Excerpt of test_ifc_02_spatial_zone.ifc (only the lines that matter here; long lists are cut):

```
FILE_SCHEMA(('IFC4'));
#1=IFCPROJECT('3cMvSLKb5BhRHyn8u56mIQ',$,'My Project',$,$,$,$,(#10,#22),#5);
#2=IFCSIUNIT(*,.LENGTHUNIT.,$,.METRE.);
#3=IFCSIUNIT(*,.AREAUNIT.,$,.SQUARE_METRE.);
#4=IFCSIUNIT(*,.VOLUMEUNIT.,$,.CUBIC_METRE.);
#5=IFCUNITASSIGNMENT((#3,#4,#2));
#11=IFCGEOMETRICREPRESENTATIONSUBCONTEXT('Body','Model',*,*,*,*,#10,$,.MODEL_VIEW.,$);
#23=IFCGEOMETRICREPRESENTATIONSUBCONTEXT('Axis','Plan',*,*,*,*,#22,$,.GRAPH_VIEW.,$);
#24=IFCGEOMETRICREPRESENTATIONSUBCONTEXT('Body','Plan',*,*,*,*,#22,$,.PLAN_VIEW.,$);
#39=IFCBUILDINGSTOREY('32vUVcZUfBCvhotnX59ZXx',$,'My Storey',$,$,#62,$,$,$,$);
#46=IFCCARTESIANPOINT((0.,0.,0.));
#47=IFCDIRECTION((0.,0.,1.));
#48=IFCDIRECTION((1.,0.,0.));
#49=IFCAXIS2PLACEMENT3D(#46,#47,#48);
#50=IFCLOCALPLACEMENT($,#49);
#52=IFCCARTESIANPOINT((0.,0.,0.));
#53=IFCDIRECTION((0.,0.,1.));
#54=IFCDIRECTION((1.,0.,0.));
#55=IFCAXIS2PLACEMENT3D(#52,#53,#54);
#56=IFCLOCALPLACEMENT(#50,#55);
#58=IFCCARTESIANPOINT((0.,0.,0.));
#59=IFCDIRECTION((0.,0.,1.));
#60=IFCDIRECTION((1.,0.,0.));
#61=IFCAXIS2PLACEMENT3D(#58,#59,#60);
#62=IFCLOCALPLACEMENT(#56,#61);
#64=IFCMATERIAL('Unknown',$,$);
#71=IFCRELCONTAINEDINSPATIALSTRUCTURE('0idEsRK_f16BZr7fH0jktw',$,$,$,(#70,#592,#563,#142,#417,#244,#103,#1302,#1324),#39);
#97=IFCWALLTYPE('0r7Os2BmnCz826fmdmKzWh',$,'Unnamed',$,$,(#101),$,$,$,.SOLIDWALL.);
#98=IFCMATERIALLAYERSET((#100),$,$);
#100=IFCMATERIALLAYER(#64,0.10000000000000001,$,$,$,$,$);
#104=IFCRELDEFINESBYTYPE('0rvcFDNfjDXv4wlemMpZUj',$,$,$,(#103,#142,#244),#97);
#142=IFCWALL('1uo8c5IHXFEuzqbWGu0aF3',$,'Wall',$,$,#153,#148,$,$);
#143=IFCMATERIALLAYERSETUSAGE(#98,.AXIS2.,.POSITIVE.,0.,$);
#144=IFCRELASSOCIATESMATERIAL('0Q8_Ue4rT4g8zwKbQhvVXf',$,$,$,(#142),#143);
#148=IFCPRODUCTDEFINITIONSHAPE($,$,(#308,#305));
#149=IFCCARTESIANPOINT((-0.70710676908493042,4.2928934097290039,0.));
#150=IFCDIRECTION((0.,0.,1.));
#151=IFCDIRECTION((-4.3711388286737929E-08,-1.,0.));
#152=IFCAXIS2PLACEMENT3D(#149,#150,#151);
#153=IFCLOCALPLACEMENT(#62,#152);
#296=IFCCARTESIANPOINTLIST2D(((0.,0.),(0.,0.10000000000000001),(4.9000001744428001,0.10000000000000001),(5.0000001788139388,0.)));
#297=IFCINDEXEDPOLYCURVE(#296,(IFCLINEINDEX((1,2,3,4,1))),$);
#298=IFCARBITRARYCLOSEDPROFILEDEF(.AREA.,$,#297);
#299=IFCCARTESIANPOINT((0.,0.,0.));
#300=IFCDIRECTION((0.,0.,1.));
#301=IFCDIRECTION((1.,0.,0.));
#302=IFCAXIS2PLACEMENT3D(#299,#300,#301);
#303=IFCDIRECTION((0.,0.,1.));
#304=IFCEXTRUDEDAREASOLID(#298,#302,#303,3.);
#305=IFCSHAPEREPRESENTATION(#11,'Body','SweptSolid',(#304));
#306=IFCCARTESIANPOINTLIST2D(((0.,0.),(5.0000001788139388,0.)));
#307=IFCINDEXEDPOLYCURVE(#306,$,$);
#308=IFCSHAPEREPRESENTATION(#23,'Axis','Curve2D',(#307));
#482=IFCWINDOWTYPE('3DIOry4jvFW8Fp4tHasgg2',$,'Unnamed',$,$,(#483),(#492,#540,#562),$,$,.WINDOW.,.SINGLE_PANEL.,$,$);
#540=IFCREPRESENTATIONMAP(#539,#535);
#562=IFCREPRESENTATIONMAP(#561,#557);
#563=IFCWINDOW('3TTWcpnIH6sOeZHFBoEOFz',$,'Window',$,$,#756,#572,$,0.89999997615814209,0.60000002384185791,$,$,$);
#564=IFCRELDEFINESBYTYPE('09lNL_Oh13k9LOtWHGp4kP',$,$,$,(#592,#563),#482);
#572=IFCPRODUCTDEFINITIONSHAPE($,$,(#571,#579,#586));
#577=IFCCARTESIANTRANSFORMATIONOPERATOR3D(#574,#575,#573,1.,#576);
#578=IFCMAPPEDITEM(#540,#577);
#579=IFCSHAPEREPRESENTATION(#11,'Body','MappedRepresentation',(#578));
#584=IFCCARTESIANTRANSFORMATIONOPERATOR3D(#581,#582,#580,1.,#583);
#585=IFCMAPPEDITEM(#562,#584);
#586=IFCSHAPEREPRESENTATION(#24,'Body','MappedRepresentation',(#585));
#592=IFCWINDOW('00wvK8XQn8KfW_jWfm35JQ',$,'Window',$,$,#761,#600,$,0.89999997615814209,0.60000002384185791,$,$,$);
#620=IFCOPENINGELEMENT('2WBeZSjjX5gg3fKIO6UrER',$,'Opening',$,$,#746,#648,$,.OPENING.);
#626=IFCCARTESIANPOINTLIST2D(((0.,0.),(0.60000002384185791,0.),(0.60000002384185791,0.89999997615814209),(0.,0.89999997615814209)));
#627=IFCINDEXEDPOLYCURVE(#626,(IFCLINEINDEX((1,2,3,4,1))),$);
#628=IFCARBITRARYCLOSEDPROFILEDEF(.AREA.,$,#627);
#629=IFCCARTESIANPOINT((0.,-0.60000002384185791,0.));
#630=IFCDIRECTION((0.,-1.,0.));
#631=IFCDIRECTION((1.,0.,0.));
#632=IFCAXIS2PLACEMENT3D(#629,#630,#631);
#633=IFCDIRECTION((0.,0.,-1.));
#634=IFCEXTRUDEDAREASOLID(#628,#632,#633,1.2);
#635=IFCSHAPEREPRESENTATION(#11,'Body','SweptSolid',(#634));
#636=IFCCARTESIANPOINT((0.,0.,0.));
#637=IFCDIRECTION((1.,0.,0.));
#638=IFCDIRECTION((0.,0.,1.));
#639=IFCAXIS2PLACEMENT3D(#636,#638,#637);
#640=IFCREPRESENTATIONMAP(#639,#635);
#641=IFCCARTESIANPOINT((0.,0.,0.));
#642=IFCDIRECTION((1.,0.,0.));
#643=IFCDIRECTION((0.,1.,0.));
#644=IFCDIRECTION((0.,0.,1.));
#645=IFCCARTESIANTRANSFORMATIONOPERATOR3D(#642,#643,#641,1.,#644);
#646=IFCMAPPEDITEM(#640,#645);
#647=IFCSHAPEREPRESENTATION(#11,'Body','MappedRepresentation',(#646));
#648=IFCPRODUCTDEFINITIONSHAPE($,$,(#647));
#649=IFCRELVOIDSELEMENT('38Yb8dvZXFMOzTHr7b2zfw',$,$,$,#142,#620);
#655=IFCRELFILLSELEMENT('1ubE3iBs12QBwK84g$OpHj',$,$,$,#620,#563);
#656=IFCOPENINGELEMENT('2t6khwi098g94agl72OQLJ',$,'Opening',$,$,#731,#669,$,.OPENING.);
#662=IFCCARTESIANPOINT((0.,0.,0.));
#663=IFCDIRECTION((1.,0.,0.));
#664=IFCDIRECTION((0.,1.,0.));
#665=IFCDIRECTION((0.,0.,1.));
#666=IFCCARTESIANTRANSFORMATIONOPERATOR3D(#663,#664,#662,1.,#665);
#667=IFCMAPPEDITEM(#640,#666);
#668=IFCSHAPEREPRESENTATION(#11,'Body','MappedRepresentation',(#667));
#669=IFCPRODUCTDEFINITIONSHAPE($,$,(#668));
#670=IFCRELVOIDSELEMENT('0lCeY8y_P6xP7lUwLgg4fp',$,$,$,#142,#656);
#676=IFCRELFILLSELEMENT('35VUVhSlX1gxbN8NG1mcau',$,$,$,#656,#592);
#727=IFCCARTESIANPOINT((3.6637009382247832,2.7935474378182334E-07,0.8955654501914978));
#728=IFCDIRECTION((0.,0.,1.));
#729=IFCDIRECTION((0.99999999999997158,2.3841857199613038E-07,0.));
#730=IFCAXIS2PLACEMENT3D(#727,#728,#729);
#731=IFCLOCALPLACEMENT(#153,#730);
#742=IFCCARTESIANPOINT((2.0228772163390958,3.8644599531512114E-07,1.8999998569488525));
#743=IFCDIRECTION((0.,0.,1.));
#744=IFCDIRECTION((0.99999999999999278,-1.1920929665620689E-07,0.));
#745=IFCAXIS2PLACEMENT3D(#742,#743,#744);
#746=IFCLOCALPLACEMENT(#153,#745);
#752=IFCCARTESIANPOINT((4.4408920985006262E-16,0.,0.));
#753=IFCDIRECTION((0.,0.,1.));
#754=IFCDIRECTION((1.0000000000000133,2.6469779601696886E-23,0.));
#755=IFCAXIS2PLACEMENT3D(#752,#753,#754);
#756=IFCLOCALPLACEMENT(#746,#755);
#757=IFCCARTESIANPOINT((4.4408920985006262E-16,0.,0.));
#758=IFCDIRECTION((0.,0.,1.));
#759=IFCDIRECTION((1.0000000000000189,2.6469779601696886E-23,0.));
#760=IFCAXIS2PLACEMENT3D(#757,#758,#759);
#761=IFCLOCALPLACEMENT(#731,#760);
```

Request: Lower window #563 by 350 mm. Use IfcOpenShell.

```python
import numpy as np
import ifcopenshell
import ifcopenshell.api.geometry
import ifcopenshell.util.placement
import ifcopenshell.util.unit

model = ifcopenshell.open("test_ifc_02_spatial_zone.ifc")
unit_scale = ifcopenshell.util.unit.calculate_unit_scale(model)

window = model.by_id(563)
opening = window.FillsVoids[0].RelatingOpeningElement
dz = -0.35 / unit_scale

shift = np.array([0.0, 0.0, dz])
# The window is placed relative to its opening, so it follows when the opening moves.
matrix = ifcopenshell.util.placement.get_local_placement(opening.ObjectPlacement)
matrix[:3, 3] += shift
ifcopenshell.api.geometry.edit_object_placement(
    model, product=opening, matrix=matrix, is_si=False, should_transform_children=True
)

print(f"moved by {dz * unit_scale:+.3f} m")

model.write("test_ifc_02_spatial_zone_edited.ifc")
```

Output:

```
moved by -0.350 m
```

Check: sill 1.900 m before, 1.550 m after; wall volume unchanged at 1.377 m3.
